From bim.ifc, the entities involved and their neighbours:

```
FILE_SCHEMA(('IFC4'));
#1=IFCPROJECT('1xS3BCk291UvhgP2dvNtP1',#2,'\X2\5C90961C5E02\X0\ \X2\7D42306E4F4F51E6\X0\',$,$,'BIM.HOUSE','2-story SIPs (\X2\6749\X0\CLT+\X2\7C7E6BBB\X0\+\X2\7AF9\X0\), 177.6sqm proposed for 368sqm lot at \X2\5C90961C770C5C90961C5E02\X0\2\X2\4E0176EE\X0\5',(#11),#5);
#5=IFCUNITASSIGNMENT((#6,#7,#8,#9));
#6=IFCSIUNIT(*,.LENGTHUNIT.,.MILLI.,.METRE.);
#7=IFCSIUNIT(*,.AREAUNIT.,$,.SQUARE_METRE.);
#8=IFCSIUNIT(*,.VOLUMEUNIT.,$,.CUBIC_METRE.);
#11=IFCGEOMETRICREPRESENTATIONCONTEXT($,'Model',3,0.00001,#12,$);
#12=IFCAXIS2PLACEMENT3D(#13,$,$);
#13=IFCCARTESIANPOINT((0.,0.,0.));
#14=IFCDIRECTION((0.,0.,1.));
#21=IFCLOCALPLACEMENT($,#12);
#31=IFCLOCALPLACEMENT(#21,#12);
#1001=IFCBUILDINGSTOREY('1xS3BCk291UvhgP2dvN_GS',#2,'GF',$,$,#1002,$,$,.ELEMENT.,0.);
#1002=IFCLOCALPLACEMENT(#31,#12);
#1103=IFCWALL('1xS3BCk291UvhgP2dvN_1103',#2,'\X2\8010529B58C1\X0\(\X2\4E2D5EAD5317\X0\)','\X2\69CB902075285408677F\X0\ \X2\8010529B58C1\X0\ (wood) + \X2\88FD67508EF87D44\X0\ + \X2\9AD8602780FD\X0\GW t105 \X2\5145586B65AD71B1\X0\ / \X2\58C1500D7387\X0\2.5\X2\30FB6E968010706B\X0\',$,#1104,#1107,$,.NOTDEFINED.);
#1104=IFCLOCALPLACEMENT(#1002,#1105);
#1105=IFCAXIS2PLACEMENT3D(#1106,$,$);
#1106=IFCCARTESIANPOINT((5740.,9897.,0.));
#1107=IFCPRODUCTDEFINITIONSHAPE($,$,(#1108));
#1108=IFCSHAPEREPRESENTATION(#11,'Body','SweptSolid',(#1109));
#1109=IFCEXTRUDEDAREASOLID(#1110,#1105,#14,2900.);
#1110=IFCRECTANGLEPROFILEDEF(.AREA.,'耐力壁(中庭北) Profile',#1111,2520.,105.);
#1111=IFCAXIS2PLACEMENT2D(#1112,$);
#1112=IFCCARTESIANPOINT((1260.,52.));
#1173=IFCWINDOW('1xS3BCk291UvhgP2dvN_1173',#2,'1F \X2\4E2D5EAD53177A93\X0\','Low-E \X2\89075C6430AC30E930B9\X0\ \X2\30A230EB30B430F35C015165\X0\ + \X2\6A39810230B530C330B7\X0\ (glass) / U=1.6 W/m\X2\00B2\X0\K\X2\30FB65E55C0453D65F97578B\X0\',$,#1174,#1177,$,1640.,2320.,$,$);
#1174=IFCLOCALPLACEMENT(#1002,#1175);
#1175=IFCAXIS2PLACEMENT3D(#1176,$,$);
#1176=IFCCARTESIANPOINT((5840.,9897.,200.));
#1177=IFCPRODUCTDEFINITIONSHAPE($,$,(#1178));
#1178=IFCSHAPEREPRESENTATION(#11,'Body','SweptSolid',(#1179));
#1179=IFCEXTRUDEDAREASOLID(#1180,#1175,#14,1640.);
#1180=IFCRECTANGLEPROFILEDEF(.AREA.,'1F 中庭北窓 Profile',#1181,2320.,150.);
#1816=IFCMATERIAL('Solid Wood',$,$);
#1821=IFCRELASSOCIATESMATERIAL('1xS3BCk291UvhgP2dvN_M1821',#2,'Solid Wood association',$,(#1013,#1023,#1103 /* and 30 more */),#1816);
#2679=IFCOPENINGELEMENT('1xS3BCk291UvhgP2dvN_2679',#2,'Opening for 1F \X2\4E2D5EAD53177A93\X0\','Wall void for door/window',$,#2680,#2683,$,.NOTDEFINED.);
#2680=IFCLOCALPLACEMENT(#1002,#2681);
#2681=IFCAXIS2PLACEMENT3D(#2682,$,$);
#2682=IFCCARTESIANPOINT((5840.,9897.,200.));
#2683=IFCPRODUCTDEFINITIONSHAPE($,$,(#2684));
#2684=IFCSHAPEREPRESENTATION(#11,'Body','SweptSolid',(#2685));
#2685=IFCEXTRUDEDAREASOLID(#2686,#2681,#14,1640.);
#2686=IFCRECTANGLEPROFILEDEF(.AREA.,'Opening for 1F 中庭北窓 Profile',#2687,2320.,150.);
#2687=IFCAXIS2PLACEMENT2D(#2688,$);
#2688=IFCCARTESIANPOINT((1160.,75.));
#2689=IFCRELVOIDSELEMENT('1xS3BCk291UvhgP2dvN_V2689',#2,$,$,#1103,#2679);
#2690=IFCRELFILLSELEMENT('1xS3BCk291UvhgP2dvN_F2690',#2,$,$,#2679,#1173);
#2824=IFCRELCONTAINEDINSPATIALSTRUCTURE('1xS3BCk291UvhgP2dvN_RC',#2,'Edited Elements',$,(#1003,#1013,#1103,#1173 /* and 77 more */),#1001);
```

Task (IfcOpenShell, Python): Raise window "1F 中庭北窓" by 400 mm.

```python
import numpy as np
import ifcopenshell
import ifcopenshell.api.geometry
import ifcopenshell.util.placement
import ifcopenshell.util.unit

model = ifcopenshell.open("bim.ifc")
unit_scale = ifcopenshell.util.unit.calculate_unit_scale(model)

window = model.by_guid("1xS3BCk291UvhgP2dvN_1173")
opening = window.FillsVoids[0].RelatingOpeningElement
dz = 400.0

shift = np.array([0.0, 0.0, dz])
# The window is not placed relative to its opening, so move both.
for product in (opening, window):
    matrix = ifcopenshell.util.placement.get_local_placement(product.ObjectPlacement)
    matrix[:3, 3] += shift
    ifcopenshell.api.geometry.edit_object_placement(model, product=product, matrix=matrix, is_si=False)

print(f"moved by {dz * unit_scale:+.3f} m")

model.write("bim_updated.ifc")
```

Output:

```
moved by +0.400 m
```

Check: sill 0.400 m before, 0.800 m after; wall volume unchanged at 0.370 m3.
